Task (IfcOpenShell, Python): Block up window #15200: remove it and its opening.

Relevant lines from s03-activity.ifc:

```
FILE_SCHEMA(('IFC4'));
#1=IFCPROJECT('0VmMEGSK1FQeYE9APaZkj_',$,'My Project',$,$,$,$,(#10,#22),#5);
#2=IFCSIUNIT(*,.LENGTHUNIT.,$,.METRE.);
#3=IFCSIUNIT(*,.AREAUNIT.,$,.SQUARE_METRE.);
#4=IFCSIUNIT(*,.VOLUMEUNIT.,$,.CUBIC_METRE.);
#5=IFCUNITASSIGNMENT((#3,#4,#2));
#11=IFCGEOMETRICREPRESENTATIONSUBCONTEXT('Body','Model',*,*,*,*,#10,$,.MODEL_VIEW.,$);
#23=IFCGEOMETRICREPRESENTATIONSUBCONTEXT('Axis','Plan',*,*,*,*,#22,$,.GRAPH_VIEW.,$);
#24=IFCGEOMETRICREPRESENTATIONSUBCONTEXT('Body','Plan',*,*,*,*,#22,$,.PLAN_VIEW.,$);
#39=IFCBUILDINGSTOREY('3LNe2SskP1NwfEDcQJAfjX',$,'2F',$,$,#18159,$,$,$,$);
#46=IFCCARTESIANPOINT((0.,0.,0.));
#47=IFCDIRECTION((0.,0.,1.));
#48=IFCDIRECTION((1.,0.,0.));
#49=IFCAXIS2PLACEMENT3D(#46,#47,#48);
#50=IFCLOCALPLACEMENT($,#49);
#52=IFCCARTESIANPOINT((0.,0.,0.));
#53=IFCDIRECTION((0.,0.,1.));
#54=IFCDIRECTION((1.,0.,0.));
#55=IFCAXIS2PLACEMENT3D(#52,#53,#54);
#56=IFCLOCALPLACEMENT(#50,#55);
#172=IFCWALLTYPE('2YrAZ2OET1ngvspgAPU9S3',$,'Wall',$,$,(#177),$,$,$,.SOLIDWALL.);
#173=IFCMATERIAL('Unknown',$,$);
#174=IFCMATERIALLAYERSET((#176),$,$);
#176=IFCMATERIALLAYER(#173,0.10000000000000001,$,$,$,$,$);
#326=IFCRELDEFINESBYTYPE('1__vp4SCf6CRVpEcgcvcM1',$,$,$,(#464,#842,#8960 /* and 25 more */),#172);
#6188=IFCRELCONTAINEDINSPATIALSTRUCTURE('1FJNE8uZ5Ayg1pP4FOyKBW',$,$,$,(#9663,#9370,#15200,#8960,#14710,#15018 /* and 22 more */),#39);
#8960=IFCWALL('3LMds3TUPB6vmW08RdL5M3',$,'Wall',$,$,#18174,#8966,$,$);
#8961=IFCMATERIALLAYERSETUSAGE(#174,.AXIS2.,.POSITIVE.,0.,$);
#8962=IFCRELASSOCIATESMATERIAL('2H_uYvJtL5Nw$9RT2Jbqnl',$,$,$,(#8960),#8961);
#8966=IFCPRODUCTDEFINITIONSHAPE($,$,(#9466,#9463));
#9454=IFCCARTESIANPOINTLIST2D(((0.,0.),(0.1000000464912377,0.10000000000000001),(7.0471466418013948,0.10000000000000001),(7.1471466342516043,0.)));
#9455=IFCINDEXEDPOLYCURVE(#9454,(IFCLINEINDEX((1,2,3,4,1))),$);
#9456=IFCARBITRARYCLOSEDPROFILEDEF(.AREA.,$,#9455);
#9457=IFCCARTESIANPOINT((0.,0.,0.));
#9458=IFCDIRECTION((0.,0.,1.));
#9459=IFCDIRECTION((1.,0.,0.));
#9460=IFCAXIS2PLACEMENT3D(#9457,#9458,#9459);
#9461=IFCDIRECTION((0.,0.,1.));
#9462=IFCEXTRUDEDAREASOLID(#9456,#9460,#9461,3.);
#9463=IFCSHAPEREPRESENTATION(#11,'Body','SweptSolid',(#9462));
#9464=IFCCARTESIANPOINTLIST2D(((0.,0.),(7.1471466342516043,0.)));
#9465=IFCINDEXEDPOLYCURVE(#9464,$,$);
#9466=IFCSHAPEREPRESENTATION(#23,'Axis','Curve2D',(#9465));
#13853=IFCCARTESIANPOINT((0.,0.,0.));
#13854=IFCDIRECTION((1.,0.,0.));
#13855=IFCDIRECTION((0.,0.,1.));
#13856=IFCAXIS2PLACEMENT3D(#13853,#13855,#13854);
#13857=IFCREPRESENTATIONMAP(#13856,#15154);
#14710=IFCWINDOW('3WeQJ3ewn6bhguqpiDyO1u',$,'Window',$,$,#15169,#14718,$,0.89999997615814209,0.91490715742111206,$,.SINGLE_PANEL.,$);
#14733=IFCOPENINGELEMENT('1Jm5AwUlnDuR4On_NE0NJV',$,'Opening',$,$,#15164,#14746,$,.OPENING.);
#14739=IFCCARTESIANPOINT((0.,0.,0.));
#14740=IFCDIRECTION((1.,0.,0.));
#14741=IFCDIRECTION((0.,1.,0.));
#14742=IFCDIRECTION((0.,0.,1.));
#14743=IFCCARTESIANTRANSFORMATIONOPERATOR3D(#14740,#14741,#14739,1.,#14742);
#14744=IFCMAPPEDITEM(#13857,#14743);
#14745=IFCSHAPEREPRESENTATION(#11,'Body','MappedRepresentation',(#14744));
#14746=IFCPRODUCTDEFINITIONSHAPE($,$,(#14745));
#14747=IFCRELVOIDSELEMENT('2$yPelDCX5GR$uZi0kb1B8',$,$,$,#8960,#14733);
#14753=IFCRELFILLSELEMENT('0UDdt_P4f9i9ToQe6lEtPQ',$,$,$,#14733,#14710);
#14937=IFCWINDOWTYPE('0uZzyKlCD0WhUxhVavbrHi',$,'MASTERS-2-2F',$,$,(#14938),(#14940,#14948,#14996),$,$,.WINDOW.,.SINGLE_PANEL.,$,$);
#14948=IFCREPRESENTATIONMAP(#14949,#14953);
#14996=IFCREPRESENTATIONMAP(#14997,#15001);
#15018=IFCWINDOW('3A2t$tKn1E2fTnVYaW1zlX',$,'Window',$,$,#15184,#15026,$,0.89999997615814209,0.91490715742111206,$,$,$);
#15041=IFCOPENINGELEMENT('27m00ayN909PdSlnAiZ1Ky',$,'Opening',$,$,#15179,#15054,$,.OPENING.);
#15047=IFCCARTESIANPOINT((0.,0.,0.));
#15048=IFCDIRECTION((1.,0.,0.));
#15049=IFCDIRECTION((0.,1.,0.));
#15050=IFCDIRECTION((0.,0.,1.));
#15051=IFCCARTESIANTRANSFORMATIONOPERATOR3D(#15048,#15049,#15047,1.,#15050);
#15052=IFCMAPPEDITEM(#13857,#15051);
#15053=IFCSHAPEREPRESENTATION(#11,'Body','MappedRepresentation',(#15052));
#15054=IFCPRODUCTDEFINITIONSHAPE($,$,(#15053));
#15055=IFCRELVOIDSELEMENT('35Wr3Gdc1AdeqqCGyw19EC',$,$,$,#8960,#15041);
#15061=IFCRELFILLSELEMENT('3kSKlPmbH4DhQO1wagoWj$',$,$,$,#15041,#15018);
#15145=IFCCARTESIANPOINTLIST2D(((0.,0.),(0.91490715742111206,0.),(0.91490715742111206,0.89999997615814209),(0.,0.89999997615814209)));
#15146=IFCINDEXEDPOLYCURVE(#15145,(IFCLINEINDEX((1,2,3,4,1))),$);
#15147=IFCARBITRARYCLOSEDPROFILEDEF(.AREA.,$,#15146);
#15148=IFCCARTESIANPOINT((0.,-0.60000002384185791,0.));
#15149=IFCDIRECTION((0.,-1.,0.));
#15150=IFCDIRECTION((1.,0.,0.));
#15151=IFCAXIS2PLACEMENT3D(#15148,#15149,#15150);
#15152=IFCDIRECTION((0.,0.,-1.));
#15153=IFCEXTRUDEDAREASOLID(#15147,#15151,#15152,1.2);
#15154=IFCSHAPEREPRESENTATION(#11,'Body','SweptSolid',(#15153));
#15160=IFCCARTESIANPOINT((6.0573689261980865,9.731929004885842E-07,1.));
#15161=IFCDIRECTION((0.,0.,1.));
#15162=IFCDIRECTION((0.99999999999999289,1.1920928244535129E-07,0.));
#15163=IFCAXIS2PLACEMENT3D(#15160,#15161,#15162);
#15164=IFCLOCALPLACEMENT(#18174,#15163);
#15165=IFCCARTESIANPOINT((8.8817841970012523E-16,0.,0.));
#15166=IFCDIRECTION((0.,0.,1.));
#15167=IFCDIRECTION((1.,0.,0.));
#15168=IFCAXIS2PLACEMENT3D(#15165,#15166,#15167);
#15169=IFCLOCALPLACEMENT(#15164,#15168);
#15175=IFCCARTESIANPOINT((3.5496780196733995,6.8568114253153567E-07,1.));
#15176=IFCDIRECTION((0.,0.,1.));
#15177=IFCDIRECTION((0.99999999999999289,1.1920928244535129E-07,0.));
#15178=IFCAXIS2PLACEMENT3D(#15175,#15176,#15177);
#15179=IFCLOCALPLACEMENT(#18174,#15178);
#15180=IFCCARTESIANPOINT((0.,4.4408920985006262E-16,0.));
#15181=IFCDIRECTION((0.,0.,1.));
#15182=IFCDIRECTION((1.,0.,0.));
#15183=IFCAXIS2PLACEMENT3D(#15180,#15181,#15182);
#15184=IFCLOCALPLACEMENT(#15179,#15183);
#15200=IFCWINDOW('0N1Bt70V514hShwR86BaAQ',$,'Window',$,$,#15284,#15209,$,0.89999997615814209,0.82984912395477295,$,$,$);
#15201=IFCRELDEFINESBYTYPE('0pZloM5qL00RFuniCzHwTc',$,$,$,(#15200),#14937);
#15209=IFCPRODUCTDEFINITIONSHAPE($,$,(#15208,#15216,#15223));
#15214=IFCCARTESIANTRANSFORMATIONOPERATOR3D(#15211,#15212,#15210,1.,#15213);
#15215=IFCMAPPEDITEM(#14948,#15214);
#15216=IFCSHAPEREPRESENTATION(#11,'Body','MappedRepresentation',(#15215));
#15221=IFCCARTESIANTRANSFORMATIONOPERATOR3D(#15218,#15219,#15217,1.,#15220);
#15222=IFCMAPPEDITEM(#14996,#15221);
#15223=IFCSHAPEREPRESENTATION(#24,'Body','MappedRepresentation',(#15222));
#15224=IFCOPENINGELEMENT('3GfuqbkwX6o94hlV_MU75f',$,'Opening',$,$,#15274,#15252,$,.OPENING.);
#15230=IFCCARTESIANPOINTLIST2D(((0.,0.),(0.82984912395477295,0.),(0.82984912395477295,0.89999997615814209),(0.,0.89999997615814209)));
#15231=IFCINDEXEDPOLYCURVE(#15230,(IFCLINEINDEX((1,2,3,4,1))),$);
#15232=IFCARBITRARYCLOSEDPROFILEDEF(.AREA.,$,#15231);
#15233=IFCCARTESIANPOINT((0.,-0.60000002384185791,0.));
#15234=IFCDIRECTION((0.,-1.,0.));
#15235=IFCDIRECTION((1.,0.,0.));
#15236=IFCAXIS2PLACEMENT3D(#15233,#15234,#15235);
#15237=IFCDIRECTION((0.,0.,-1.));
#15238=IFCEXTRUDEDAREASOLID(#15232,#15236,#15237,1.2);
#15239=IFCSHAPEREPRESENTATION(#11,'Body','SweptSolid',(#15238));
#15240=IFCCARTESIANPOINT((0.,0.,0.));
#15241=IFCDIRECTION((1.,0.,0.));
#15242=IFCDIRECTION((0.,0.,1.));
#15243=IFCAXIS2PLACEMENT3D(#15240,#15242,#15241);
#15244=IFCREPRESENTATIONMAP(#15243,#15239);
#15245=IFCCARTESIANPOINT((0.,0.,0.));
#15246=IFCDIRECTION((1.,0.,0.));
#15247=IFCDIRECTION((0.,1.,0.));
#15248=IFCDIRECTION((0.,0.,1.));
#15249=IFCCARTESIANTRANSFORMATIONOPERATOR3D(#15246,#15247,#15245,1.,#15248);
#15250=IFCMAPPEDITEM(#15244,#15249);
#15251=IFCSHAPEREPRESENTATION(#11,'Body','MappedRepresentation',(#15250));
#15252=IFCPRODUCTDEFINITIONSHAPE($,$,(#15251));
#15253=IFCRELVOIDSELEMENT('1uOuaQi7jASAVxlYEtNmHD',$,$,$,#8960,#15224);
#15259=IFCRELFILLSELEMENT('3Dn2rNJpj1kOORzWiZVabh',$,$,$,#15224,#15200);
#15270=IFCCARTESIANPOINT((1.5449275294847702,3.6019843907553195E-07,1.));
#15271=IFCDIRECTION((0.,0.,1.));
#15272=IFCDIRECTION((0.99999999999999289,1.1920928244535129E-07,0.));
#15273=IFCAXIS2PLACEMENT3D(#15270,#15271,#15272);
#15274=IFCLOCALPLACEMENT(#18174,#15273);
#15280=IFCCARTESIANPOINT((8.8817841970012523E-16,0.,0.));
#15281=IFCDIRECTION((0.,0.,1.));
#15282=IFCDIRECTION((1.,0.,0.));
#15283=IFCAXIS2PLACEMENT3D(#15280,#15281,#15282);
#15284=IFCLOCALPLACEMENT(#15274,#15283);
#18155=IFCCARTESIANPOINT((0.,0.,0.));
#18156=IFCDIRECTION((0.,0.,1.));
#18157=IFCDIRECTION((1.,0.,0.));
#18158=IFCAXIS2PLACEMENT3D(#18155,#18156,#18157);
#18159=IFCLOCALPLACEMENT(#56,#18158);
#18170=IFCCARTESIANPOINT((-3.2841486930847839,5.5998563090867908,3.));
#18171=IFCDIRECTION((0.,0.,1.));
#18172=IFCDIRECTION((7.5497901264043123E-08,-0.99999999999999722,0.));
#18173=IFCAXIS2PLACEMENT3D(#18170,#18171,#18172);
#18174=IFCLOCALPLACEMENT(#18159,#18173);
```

```python
import ifcopenshell
import ifcopenshell.api.feature
import ifcopenshell.api.root
import ifcopenshell.geom
import ifcopenshell.util.shape

model = ifcopenshell.open("s03-activity.ifc")
settings = ifcopenshell.geom.settings()


def volume(element):
    """Net volume in cubic metres, openings subtracted."""
    shape = ifcopenshell.geom.create_shape(settings, element)
    return ifcopenshell.util.shape.get_volume(shape.geometry)


window = model.by_id(15200)
opening = window.FillsVoids[0].RelatingOpeningElement
wall = opening.VoidsElements[0].RelatingBuildingElement
before = volume(wall)

ifcopenshell.api.root.remove_product(model, product=window)
ifcopenshell.api.feature.remove_feature(model, feature=opening)

after = volume(wall)

print(f"wall volume {before:.3f} -> {after:.3f} m3")

model.write("s03-activity-out.ifc")
```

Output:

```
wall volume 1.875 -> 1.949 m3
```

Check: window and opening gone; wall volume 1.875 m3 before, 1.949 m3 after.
